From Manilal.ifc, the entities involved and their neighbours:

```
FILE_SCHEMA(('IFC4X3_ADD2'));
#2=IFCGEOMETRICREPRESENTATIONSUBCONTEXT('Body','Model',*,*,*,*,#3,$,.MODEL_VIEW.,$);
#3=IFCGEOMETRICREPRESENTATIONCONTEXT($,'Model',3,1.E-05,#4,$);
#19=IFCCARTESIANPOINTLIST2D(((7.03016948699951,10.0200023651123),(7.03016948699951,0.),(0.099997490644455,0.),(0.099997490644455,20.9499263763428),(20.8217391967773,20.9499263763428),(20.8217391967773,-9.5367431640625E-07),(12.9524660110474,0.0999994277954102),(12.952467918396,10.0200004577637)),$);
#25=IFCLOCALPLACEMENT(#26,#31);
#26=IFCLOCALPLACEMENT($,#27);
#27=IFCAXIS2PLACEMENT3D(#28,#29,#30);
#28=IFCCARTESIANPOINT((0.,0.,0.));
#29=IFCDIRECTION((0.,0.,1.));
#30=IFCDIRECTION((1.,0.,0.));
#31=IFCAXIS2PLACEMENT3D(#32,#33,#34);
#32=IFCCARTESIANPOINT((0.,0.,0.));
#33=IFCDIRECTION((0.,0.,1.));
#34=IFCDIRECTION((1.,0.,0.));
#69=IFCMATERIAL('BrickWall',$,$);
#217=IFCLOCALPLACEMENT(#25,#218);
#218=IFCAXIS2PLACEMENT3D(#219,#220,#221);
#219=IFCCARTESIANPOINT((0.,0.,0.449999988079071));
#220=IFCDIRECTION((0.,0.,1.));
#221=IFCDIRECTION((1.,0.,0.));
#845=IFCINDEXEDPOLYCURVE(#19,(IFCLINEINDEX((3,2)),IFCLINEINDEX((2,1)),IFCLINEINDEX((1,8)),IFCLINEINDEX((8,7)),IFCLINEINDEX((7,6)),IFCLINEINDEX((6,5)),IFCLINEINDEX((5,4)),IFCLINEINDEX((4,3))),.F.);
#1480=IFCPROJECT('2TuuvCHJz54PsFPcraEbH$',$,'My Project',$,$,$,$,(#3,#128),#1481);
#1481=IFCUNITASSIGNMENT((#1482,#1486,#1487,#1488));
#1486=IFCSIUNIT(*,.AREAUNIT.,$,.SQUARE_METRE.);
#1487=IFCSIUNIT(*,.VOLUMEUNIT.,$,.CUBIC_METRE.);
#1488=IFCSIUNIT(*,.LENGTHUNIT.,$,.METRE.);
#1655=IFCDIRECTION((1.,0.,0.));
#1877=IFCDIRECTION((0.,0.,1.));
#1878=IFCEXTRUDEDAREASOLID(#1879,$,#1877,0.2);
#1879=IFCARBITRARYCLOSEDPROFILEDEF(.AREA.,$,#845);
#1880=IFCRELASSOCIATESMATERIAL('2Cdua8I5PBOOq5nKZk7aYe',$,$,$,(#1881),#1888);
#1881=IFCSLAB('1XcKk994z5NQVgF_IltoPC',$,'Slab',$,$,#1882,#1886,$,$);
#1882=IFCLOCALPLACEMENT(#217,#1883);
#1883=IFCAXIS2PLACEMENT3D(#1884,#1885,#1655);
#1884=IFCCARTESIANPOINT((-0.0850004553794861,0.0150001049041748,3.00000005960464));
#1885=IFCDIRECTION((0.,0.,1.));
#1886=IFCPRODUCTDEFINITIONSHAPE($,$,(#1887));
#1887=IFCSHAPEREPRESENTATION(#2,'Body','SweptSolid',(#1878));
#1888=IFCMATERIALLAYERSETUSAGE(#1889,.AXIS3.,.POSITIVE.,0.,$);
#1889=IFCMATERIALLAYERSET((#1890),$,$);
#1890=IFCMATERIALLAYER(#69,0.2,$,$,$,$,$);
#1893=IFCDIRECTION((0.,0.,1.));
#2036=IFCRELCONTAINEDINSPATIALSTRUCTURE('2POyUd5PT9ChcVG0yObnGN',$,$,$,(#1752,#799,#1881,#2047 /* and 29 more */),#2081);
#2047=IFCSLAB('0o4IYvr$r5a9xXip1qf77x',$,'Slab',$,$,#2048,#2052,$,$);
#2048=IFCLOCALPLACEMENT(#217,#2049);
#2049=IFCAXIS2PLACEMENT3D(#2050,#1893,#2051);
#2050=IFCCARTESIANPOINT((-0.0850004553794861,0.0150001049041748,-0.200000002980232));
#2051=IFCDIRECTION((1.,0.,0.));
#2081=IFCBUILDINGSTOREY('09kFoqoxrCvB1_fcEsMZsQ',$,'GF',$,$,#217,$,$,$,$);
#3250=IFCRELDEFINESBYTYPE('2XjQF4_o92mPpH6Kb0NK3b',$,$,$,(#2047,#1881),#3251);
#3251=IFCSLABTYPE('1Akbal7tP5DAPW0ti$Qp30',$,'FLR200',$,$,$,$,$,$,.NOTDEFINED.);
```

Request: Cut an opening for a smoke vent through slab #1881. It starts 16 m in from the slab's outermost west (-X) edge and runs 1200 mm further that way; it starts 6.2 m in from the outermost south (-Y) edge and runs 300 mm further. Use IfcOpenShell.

```python
import numpy as np
import ifcopenshell
import ifcopenshell.api.feature
import ifcopenshell.api.geometry
import ifcopenshell.api.root
import ifcopenshell.geom
import ifcopenshell.util.placement
import ifcopenshell.util.representation
import ifcopenshell.util.shape
import ifcopenshell.util.unit

model = ifcopenshell.open("Manilal.ifc")
unit_scale = ifcopenshell.util.unit.calculate_unit_scale(model)
settings = ifcopenshell.geom.settings()


def volume(element):
    """Net volume in cubic metres, openings subtracted."""
    shape = ifcopenshell.geom.create_shape(settings, element)
    return ifcopenshell.util.shape.get_volume(shape.geometry)


slab = model.by_guid("1XcKk994z5NQVgF_IltoPC")
before = volume(slab)

# Extent in the slab's own axes, in metres. The edges named are its -X and -Y sides.
slab_shape = ifcopenshell.geom.create_shape(settings, slab)
vertices = ifcopenshell.util.shape.get_vertices(slab_shape.geometry)
x_min, y_min, bottom = vertices.min(axis=0)
top = vertices[:, 2].max()

opening = ifcopenshell.api.root.create_entity(model, ifc_class="IfcOpeningElement", name="Smoke vent opening", predefined_type="OPENING")
context = ifcopenshell.util.representation.get_context(model, "Model", "Body", "MODEL_VIEW")
width, depth = 1.2, 0.3
outline = [(0.0, 0.0), (width, 0.0), (width, depth), (0.0, depth), (0.0, 0.0)]
# Overshoot both faces by 50 mm so the cut is clean.
shape = ifcopenshell.api.geometry.add_slab_representation(
    model, context=context, depth=top - bottom + 0.1, polyline=outline
)
ifcopenshell.api.geometry.assign_representation(model, product=opening, representation=shape)

matrix = ifcopenshell.util.placement.get_local_placement(slab.ObjectPlacement)
matrix[:, 3] = matrix @ np.append(np.array([x_min + 16, y_min + 6.2, bottom - 0.05]) / unit_scale, 1.0)
ifcopenshell.api.geometry.edit_object_placement(model, product=opening, matrix=matrix, is_si=False)
ifcopenshell.api.feature.add_feature(model, feature=opening, element=slab)

after = volume(slab)

print(f"slab volume {before:.3f} -> {after:.3f} m3")

model.write("Manilal-out.ifc")
```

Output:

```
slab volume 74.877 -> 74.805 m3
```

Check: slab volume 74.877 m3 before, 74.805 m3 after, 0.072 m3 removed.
